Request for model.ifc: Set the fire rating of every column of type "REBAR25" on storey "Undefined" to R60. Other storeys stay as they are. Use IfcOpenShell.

First a look at what the model holds.

```python
import ifcopenshell
import ifcopenshell.util.element

model = ifcopenshell.open("model.ifc")
print(model.schema)
storey = next(s for s in model.by_type("IfcBuildingStorey") if s.Name == "Undefined")
columns = [e for e in ifcopenshell.util.element.get_decomposition(storey) if e.is_a("IfcColumn")]
seen = {}
for e in columns:
    element_type = ifcopenshell.util.element.get_type(e)
    key = (element_type.Name if element_type != e and element_type else None, ifcopenshell.util.element.get_pset(e, "Pset_ColumnCommon", "FireRating"))
    seen[key] = seen.get(key, 0) + 1
for (name, value), count in sorted(seen.items(), key=str):
    print(count, "x", name, "|", value)
```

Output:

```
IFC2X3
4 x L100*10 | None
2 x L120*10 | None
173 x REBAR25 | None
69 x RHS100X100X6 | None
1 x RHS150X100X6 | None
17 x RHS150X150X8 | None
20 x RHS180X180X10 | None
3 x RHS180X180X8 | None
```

```python
import ifcopenshell
import ifcopenshell.api.pset
import ifcopenshell.util.element

model = ifcopenshell.open("model.ifc")

storey = next(s for s in model.by_type("IfcBuildingStorey") if s.Name == "Undefined")
columns = [e for e in ifcopenshell.util.element.get_decomposition(storey) if e.is_a("IfcColumn")]

count = 0
for e in columns:
    element_type = ifcopenshell.util.element.get_type(e)
    if element_type in (None, e) or element_type.Name != "REBAR25":
        continue
    found = ifcopenshell.util.element.get_pset(e, "Pset_ColumnCommon", should_inherit=False)
    if found:
        pset = model.by_id(found["id"])
        if len(ifcopenshell.util.element.get_elements_by_pset(pset)) > 1:
            pset = ifcopenshell.api.pset.unshare_pset(model, products=[e], pset=pset)[0]
    else:
        pset = ifcopenshell.api.pset.add_pset(model, product=e, name="Pset_ColumnCommon")
    ifcopenshell.api.pset.edit_pset(model, pset=pset, properties={"FireRating": "R60"})
    count += 1

print(count, "columns updated")

model.write("model_updated.ifc")
```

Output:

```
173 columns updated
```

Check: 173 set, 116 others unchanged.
